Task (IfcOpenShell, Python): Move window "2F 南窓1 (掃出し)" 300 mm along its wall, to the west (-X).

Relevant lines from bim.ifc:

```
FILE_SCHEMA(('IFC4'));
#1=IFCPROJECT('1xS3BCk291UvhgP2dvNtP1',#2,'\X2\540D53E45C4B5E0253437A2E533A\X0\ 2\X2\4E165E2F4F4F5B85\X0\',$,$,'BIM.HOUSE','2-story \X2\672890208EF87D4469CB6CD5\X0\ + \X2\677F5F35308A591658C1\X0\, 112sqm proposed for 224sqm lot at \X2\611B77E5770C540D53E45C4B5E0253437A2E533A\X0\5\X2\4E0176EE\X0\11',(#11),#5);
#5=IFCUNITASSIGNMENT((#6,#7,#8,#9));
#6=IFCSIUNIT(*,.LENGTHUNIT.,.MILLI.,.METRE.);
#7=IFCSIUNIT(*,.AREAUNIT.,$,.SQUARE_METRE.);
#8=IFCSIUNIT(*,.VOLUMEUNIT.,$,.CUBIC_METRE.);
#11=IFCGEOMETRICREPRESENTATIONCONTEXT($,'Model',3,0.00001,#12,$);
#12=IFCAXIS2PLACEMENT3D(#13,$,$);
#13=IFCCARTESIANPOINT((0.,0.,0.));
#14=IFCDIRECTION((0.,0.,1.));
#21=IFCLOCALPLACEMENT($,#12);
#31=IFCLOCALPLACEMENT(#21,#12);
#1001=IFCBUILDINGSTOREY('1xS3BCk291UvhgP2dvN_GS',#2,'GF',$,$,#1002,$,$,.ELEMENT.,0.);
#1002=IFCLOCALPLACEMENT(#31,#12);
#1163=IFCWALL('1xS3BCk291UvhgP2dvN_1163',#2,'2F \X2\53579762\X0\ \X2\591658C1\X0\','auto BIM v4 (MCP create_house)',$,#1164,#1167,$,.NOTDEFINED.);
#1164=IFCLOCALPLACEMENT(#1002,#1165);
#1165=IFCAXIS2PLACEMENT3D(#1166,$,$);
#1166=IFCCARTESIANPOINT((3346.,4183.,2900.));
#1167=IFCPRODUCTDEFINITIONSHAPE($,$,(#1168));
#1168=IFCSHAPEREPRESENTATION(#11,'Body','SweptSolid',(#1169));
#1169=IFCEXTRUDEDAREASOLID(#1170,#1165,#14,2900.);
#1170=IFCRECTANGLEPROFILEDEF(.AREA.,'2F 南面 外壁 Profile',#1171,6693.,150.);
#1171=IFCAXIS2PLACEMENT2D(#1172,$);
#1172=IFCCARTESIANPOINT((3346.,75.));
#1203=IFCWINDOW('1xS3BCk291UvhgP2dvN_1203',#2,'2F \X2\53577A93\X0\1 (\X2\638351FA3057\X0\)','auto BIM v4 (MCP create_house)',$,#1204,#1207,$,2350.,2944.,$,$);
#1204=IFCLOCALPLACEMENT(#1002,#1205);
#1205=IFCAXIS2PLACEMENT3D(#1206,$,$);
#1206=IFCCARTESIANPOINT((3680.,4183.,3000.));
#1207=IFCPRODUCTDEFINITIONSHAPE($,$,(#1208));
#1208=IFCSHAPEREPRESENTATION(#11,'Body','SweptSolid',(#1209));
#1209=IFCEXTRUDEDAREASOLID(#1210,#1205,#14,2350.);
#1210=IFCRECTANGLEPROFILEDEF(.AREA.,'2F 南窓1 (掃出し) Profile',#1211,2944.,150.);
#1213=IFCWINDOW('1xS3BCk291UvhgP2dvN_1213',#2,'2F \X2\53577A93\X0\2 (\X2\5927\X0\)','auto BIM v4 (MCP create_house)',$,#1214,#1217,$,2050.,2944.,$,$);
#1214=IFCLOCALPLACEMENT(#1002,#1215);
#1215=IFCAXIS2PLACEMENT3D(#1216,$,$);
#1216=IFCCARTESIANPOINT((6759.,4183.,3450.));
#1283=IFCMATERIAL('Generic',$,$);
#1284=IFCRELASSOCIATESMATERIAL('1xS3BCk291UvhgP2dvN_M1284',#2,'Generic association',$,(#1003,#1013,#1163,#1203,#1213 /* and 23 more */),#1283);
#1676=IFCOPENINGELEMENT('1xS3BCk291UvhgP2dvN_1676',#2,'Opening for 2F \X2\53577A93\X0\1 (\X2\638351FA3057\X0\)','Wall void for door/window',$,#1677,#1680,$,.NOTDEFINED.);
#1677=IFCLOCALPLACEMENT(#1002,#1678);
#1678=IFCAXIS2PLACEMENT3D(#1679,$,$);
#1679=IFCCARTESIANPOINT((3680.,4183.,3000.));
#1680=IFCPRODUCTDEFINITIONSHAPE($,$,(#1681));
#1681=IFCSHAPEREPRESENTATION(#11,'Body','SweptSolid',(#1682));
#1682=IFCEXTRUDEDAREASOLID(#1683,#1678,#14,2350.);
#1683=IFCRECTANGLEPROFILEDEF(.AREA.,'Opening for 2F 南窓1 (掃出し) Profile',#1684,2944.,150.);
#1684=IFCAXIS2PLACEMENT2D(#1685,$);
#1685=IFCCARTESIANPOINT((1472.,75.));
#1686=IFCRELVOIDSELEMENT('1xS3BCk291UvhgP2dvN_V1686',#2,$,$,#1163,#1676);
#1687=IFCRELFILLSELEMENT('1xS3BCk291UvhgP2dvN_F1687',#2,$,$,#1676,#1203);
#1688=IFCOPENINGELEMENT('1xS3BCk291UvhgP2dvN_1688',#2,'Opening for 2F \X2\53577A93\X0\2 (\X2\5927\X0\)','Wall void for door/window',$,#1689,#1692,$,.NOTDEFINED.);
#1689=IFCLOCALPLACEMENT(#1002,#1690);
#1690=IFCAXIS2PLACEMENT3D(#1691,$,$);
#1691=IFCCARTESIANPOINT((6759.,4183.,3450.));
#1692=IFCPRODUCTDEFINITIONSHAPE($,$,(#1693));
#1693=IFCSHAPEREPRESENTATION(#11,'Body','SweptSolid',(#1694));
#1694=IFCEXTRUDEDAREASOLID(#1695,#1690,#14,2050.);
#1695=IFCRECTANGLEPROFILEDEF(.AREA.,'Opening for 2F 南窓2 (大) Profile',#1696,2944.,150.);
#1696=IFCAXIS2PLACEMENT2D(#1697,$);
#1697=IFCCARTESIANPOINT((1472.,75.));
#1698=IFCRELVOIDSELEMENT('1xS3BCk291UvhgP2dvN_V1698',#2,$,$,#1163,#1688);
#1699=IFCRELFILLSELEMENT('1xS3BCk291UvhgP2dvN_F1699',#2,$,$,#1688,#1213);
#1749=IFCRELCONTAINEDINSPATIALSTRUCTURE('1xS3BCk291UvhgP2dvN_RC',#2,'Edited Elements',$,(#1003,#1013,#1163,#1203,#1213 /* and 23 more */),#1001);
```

```python
import ifcopenshell
import ifcopenshell.api.geometry
import ifcopenshell.util.placement
import ifcopenshell.util.unit

model = ifcopenshell.open("bim.ifc")
unit_scale = ifcopenshell.util.unit.calculate_unit_scale(model)

window = model.by_guid("1xS3BCk291UvhgP2dvN_1203")
opening = window.FillsVoids[0].RelatingOpeningElement
wall = opening.VoidsElements[0].RelatingBuildingElement

wall_matrix = ifcopenshell.util.placement.get_local_placement(wall.ObjectPlacement)
shift = wall_matrix[:3, 0] * -0.3 / unit_scale
before = ifcopenshell.util.placement.get_local_placement(window.ObjectPlacement)[:3, 3].copy()

# The window is not placed relative to its opening, so move both.
for product in (opening, window):
    matrix = ifcopenshell.util.placement.get_local_placement(product.ObjectPlacement)
    matrix[:3, 3] += shift
    ifcopenshell.api.geometry.edit_object_placement(model, product=product, matrix=matrix, is_si=False)

after = ifcopenshell.util.placement.get_local_placement(window.ObjectPlacement)[:3, 3]
print("window moved by", (after - before).round(3) + 0.0)

model.write("bim_v2.ifc")
```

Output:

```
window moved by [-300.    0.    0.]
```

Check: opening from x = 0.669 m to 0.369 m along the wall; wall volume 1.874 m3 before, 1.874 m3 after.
